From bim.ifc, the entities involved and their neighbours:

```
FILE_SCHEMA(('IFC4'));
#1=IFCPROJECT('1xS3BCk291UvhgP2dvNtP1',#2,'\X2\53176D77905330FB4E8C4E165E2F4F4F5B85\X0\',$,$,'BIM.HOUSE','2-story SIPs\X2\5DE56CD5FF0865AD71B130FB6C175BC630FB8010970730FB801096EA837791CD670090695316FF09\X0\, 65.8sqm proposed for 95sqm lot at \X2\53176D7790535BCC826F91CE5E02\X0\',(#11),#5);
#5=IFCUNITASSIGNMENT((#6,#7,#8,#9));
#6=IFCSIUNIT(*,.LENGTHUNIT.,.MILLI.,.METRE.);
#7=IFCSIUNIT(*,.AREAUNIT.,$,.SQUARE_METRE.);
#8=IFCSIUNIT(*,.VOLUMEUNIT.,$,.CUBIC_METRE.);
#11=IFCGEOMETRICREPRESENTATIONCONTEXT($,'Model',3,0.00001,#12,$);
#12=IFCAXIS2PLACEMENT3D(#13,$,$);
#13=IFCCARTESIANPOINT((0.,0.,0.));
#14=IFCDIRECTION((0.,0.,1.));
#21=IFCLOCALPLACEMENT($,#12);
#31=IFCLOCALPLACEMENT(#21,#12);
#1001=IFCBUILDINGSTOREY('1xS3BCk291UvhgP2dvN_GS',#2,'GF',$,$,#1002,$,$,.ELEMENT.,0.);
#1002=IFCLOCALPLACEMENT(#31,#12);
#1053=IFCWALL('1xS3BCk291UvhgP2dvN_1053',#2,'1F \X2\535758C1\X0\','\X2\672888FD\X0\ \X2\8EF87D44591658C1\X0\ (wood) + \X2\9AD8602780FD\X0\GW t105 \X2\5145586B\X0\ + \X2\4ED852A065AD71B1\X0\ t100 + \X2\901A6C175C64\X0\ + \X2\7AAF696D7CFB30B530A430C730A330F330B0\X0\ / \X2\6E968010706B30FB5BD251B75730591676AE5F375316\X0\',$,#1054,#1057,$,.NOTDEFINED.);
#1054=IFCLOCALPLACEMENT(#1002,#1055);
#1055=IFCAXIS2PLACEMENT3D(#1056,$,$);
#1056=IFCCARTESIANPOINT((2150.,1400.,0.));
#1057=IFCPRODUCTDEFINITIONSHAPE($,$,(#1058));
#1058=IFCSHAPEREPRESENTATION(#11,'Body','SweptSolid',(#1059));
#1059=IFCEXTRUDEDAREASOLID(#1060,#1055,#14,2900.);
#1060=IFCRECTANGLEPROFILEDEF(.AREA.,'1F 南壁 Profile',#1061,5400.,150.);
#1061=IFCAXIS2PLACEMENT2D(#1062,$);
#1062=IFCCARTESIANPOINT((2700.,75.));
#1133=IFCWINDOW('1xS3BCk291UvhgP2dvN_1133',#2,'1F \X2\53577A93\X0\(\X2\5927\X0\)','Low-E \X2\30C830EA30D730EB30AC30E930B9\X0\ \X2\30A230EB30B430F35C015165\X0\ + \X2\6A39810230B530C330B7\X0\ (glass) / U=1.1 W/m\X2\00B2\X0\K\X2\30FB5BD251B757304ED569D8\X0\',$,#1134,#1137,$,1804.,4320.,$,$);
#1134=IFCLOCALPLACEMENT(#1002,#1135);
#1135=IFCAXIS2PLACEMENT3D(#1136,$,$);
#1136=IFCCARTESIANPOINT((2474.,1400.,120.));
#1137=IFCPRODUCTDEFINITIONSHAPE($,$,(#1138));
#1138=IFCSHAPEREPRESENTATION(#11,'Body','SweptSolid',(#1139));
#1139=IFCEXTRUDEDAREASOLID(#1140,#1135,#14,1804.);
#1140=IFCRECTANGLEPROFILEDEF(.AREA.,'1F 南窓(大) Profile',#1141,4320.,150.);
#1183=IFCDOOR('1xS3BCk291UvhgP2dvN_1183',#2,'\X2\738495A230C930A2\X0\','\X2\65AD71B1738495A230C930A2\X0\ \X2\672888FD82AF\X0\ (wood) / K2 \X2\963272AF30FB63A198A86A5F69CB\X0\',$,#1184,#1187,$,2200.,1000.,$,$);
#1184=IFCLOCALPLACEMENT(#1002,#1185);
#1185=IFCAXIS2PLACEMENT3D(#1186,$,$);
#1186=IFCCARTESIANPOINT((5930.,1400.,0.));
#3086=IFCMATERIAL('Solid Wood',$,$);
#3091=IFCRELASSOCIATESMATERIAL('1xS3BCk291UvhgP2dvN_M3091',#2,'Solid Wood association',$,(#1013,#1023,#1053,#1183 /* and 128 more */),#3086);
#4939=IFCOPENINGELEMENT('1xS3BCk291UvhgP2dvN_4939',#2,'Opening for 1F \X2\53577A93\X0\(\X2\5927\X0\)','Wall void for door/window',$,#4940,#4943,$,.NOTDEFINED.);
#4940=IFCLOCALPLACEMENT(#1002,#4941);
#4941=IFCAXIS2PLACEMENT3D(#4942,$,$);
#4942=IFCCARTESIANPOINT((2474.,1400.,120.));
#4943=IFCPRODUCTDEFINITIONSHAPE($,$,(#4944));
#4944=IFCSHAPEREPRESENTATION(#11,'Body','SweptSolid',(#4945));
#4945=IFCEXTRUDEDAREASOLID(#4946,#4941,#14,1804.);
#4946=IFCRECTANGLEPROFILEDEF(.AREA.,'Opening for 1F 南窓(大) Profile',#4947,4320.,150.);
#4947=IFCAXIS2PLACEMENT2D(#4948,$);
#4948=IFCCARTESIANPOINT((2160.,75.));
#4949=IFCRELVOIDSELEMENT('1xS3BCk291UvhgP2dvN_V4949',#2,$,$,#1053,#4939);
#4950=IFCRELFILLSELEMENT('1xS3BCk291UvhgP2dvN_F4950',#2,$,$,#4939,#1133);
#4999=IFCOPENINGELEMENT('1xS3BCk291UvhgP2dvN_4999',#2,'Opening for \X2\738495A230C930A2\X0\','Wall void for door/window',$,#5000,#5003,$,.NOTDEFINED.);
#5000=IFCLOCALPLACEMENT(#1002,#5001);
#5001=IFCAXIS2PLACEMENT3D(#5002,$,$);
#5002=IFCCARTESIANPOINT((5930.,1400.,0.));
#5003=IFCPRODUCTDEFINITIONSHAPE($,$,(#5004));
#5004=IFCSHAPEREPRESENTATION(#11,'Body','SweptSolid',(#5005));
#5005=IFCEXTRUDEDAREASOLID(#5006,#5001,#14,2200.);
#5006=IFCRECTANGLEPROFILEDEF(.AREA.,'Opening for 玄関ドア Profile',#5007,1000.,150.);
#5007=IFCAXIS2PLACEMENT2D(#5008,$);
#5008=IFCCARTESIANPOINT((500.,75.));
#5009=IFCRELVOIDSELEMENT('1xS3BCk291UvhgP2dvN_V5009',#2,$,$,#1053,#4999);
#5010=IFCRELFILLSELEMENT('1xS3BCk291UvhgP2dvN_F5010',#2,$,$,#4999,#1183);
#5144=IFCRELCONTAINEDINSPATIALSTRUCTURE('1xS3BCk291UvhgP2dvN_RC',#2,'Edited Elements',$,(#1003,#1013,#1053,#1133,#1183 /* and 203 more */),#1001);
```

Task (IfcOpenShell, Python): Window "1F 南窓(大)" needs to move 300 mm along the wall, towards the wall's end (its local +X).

```python
import ifcopenshell
import ifcopenshell.api.geometry
import ifcopenshell.util.placement
import ifcopenshell.util.unit

model = ifcopenshell.open("bim.ifc")
unit_scale = ifcopenshell.util.unit.calculate_unit_scale(model)

window = model.by_guid("1xS3BCk291UvhgP2dvN_1133")
opening = window.FillsVoids[0].RelatingOpeningElement
wall = opening.VoidsElements[0].RelatingBuildingElement

wall_matrix = ifcopenshell.util.placement.get_local_placement(wall.ObjectPlacement)
shift = wall_matrix[:3, 0] * 0.3 / unit_scale
before = ifcopenshell.util.placement.get_local_placement(window.ObjectPlacement)[:3, 3].copy()

# The window is not placed relative to its opening, so move both.
for product in (opening, window):
    matrix = ifcopenshell.util.placement.get_local_placement(product.ObjectPlacement)
    matrix[:3, 3] += shift
    ifcopenshell.api.geometry.edit_object_placement(model, product=product, matrix=matrix, is_si=False)

after = ifcopenshell.util.placement.get_local_placement(window.ObjectPlacement)[:3, 3]
print("window moved by", (after - before).round(3) + 0.0)

model.write("bim_rev.ifc")
```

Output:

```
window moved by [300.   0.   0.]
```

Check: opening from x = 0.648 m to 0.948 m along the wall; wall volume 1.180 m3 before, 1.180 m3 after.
